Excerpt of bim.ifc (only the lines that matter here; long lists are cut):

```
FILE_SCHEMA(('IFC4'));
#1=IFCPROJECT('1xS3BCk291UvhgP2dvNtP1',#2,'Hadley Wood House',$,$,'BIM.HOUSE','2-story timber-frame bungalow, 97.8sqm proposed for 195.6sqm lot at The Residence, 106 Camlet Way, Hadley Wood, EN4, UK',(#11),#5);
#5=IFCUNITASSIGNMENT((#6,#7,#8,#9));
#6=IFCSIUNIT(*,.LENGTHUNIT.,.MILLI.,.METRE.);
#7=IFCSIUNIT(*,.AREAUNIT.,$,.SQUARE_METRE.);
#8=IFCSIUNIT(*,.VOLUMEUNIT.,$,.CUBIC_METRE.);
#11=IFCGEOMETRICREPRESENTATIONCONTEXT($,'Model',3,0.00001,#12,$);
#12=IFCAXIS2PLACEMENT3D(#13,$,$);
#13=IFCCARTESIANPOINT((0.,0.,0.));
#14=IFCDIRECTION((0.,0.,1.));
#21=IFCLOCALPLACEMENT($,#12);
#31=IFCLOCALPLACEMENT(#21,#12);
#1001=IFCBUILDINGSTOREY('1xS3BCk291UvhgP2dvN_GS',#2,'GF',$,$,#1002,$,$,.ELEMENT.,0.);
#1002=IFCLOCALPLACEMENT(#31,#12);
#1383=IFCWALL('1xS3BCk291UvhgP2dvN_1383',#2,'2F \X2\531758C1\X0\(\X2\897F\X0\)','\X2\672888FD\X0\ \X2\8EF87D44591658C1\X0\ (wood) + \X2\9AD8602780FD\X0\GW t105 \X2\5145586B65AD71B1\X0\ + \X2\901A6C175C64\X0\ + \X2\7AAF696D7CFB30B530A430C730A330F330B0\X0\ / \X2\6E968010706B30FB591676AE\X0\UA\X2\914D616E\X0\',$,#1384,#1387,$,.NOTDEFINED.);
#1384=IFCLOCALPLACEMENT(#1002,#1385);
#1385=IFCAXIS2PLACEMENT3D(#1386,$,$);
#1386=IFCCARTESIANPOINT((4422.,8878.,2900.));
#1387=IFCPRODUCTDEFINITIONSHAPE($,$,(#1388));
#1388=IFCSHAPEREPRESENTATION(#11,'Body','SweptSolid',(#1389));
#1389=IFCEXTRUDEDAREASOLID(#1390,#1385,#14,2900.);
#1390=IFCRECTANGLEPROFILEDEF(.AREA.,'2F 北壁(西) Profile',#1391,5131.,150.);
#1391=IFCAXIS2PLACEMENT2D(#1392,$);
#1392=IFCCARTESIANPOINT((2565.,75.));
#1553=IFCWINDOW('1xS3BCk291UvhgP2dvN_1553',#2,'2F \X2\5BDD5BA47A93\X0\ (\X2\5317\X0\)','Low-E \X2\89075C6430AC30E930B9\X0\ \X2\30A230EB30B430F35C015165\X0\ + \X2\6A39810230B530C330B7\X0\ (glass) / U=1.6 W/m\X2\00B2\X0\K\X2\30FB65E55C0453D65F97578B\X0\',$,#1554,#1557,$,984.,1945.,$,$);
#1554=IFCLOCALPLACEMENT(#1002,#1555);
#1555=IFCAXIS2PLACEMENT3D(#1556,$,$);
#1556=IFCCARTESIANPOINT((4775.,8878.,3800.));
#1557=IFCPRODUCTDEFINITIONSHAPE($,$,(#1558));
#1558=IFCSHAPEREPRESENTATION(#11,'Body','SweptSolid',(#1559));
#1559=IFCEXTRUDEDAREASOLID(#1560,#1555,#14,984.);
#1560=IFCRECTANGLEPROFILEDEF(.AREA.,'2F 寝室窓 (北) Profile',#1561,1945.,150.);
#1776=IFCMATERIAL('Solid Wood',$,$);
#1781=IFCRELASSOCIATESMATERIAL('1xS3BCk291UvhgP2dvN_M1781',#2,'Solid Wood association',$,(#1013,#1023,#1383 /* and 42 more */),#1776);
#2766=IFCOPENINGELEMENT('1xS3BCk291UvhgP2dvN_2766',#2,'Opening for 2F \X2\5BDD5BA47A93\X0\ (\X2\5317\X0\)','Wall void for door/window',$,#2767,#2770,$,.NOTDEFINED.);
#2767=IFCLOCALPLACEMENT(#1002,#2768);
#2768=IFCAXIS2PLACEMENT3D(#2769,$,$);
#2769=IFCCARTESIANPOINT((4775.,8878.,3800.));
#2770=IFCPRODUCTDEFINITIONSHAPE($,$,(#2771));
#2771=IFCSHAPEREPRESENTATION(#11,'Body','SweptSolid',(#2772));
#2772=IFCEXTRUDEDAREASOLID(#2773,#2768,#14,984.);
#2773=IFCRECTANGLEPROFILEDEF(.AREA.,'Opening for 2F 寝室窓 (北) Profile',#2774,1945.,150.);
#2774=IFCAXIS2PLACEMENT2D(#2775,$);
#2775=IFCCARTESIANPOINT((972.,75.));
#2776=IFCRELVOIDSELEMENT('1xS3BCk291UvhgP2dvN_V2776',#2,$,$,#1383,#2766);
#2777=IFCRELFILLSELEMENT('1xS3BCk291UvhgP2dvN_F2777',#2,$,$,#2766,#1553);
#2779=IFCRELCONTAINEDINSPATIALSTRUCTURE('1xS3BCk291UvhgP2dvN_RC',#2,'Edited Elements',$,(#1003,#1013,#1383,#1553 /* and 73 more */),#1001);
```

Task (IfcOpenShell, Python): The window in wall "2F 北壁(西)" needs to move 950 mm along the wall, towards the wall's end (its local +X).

```python
import ifcopenshell
import ifcopenshell.api.geometry
import ifcopenshell.util.placement
import ifcopenshell.util.unit

model = ifcopenshell.open("bim.ifc")
unit_scale = ifcopenshell.util.unit.calculate_unit_scale(model)

window = model.by_guid("1xS3BCk291UvhgP2dvN_1553")
opening = window.FillsVoids[0].RelatingOpeningElement
wall = opening.VoidsElements[0].RelatingBuildingElement

wall_matrix = ifcopenshell.util.placement.get_local_placement(wall.ObjectPlacement)
shift = wall_matrix[:3, 0] * 0.95 / unit_scale
before = ifcopenshell.util.placement.get_local_placement(window.ObjectPlacement)[:3, 3].copy()

# The window is not placed relative to its opening, so move both.
for product in (opening, window):
    matrix = ifcopenshell.util.placement.get_local_placement(product.ObjectPlacement)
    matrix[:3, 3] += shift
    ifcopenshell.api.geometry.edit_object_placement(model, product=product, matrix=matrix, is_si=False)

after = ifcopenshell.util.placement.get_local_placement(window.ObjectPlacement)[:3, 3]
print("window moved by", (after - before).round(3) + 0.0)

model.write("bim_updated.ifc")
```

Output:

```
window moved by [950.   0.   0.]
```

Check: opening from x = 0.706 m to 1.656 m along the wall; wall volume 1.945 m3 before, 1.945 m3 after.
